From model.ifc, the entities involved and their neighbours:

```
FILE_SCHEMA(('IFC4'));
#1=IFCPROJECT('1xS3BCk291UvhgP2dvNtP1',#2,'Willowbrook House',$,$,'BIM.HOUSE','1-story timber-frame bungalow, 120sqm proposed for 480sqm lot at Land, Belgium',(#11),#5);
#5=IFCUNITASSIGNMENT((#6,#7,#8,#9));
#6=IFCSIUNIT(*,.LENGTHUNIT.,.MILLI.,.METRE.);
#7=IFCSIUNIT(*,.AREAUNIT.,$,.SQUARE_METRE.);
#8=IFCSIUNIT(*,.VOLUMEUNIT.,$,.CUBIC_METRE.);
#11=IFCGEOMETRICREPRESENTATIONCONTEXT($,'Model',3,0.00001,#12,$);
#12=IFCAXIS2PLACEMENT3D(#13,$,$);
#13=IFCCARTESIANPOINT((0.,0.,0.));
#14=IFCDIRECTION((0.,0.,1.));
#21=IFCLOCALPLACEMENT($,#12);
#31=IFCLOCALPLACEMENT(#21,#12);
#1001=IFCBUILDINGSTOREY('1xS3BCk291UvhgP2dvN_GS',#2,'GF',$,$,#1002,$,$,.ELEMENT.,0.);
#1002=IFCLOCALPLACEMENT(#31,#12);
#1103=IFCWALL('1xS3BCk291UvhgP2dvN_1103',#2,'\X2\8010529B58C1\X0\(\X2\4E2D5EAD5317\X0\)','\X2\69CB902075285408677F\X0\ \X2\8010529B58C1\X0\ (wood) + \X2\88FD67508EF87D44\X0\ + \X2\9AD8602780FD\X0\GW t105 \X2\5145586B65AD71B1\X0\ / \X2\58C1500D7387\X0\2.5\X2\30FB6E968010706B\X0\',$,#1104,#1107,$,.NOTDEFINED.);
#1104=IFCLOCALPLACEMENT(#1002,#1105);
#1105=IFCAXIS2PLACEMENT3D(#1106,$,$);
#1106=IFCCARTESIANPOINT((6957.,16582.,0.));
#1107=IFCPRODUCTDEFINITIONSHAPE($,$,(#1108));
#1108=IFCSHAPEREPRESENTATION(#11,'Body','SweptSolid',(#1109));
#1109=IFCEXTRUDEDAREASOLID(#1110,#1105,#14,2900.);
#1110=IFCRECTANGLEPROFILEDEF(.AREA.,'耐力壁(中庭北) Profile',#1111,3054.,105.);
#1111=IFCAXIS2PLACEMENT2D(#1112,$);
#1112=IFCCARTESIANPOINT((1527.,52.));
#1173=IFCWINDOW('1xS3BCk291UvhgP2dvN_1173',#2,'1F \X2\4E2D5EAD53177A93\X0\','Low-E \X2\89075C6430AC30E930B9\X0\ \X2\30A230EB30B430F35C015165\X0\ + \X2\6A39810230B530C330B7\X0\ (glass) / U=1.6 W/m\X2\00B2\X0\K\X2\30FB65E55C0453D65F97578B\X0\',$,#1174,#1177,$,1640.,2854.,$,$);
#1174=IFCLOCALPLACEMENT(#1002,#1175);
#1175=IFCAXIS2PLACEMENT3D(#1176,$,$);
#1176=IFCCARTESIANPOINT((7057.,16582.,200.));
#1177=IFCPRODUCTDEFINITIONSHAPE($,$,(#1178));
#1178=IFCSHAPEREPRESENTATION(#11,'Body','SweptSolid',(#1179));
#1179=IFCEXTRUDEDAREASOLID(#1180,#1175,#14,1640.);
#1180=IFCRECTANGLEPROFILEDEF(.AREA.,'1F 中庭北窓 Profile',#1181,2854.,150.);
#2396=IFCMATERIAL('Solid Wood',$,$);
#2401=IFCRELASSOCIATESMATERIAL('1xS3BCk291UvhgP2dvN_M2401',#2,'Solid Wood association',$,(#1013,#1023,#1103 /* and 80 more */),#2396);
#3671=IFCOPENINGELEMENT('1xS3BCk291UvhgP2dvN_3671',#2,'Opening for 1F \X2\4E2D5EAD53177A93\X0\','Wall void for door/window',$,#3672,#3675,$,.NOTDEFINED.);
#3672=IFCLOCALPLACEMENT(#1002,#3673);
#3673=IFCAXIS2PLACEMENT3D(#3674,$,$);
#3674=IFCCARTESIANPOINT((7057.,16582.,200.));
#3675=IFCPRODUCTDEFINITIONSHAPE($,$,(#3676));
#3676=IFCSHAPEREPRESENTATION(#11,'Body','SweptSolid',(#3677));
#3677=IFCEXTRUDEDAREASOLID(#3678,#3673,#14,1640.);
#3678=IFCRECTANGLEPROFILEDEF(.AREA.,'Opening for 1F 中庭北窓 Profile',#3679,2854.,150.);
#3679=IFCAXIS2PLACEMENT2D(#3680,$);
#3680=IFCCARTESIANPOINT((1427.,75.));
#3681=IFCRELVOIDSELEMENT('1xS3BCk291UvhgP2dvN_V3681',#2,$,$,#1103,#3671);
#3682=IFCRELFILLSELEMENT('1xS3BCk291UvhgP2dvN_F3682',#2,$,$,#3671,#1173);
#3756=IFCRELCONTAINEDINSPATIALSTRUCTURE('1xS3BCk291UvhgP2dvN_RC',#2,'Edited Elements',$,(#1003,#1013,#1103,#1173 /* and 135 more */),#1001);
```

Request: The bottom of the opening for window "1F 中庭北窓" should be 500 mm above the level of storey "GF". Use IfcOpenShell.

```python
import numpy as np
import ifcopenshell
import ifcopenshell.api.geometry
import ifcopenshell.geom
import ifcopenshell.util.element
import ifcopenshell.util.placement
import ifcopenshell.util.shape
import ifcopenshell.util.unit

model = ifcopenshell.open("model.ifc")
unit_scale = ifcopenshell.util.unit.calculate_unit_scale(model)

window = model.by_guid("1xS3BCk291UvhgP2dvN_1173")
opening = window.FillsVoids[0].RelatingOpeningElement
storey = ifcopenshell.util.element.get_container(window, ifc_class="IfcBuildingStorey")
level = ifcopenshell.util.placement.get_local_placement(storey.ObjectPlacement)[2, 3]

# The opening's origin need not be at the sill, so measure its lowest point.
shape = ifcopenshell.geom.create_shape(ifcopenshell.geom.settings(), opening)
bottom = ifcopenshell.util.shape.get_shape_bottom_elevation(shape, shape.geometry) / unit_scale
dz = level + 0.5 / unit_scale - bottom

shift = np.array([0.0, 0.0, dz])
# The window is not placed relative to its opening, so move both.
for product in (opening, window):
    matrix = ifcopenshell.util.placement.get_local_placement(product.ObjectPlacement)
    matrix[:3, 3] += shift
    ifcopenshell.api.geometry.edit_object_placement(model, product=product, matrix=matrix, is_si=False)

print(f"moved by {dz * unit_scale:+.3f} m")

model.write("model_rev.ifc")
```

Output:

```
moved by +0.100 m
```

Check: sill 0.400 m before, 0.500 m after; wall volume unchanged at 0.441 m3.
